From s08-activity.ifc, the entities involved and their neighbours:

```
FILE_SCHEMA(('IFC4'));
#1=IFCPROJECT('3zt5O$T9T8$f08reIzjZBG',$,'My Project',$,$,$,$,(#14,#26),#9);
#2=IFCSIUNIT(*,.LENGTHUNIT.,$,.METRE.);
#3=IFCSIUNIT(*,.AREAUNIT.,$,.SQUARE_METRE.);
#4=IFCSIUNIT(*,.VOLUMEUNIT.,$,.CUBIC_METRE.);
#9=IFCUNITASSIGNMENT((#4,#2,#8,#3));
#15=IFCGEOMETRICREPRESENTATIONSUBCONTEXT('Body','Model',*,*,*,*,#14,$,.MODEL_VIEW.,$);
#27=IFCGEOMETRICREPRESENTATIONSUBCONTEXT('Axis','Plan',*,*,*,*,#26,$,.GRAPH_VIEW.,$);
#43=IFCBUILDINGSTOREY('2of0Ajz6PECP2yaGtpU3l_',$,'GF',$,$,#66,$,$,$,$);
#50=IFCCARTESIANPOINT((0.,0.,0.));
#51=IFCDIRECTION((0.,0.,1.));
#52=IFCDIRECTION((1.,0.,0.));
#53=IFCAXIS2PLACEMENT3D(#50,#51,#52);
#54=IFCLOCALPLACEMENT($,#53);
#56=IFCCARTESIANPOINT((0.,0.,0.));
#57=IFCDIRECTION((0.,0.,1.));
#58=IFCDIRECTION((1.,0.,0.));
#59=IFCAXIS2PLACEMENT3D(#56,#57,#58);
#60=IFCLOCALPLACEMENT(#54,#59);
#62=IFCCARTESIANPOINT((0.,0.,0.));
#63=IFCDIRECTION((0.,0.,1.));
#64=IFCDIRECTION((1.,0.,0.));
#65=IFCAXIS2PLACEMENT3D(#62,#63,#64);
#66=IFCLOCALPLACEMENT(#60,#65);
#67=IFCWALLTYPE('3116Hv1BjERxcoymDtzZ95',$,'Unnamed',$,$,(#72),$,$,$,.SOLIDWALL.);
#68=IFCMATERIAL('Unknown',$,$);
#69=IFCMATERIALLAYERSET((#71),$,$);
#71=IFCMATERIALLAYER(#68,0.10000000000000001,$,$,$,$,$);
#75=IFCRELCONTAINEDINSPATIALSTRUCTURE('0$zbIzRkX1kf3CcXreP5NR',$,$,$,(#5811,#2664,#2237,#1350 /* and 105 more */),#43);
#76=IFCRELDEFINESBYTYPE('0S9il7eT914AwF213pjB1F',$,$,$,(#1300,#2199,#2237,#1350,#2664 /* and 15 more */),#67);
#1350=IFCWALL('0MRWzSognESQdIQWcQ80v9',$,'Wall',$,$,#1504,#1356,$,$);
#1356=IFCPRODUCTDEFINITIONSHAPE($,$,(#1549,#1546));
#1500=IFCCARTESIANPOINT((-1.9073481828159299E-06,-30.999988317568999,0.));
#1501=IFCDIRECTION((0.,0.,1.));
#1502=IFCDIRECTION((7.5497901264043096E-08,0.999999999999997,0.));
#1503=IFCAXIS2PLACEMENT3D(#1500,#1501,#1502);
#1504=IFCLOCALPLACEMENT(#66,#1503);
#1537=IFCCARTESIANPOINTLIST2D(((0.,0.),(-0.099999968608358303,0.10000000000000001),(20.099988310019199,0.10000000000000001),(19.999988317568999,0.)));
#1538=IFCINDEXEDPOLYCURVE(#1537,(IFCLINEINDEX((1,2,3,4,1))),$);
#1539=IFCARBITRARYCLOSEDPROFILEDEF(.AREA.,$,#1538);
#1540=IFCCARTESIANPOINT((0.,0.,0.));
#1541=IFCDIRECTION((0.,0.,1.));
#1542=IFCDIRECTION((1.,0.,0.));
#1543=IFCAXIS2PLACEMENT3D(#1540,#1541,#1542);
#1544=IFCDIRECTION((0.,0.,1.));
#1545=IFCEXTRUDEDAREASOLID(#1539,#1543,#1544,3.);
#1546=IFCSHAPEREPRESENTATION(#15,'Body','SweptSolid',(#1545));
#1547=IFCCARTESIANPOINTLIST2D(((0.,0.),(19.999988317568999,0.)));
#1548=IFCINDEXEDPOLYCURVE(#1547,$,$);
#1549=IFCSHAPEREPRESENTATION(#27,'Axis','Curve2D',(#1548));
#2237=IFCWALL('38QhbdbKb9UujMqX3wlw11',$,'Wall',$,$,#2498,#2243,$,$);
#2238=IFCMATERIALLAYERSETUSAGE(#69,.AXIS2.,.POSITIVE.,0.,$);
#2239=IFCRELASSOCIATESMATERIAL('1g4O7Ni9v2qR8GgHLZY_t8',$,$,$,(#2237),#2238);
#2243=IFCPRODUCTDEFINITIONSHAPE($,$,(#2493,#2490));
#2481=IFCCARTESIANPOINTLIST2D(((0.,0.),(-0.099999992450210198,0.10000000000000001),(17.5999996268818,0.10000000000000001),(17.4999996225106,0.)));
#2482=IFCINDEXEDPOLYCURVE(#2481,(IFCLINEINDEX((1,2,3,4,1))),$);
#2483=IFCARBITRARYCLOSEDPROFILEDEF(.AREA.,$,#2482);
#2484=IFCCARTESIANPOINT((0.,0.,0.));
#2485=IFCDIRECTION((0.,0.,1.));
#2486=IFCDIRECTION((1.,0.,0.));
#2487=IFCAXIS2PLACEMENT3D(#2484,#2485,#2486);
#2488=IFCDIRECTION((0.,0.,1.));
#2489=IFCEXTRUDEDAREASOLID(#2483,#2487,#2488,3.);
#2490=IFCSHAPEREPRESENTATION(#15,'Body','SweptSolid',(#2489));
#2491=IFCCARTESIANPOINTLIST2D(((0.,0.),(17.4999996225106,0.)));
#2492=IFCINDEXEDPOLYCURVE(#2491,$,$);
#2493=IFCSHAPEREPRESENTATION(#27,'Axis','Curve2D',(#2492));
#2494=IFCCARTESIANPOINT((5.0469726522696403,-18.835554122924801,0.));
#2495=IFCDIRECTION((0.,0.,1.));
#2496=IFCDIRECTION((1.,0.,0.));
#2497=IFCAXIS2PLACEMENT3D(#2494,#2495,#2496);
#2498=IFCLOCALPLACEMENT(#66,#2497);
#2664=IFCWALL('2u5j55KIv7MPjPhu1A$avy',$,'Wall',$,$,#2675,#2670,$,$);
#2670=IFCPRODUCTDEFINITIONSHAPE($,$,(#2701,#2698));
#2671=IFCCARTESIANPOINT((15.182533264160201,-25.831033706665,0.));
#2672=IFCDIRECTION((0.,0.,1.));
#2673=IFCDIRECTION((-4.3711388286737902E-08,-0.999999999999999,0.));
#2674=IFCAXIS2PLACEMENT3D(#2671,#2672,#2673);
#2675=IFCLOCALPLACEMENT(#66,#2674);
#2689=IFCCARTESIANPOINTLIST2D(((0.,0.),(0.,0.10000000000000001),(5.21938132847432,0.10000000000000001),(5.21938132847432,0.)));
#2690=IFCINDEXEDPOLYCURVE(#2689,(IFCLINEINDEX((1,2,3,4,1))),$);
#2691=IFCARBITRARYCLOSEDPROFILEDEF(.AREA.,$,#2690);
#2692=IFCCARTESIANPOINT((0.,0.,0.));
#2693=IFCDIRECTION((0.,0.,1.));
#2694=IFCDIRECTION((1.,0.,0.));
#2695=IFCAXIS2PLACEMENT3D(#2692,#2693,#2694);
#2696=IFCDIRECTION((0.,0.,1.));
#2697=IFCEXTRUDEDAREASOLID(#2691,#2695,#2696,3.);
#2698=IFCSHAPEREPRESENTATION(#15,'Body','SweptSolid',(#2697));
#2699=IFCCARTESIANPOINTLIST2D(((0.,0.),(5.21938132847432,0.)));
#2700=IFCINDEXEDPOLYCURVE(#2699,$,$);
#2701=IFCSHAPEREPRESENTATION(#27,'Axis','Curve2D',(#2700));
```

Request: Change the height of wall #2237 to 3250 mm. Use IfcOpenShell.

```python
import ifcopenshell
import ifcopenshell.geom
import ifcopenshell.util.representation
import ifcopenshell.util.shape
import ifcopenshell.util.unit

model = ifcopenshell.open("s08-activity.ifc")
unit_scale = ifcopenshell.util.unit.calculate_unit_scale(model)
settings = ifcopenshell.geom.settings()


def volume(element):
    """Net volume in cubic metres, openings subtracted."""
    shape = ifcopenshell.geom.create_shape(settings, element)
    return ifcopenshell.util.shape.get_volume(shape.geometry)


wall = model.by_guid("38QhbdbKb9UujMqX3wlw11")
before = volume(wall)

body = ifcopenshell.util.representation.get_representation(wall, "Model", "Body")
solid = body.Items[0]
old_height = solid.Depth
solid.Depth = 3.25 / unit_scale
after = volume(wall)

print(f"height {old_height:g} -> {solid.Depth:g}, volume {before:.3f} -> {after:.3f} m3")

model.write("s08-activity-out.ifc")
```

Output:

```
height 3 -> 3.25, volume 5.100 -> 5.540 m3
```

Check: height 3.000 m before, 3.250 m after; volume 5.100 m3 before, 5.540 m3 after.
